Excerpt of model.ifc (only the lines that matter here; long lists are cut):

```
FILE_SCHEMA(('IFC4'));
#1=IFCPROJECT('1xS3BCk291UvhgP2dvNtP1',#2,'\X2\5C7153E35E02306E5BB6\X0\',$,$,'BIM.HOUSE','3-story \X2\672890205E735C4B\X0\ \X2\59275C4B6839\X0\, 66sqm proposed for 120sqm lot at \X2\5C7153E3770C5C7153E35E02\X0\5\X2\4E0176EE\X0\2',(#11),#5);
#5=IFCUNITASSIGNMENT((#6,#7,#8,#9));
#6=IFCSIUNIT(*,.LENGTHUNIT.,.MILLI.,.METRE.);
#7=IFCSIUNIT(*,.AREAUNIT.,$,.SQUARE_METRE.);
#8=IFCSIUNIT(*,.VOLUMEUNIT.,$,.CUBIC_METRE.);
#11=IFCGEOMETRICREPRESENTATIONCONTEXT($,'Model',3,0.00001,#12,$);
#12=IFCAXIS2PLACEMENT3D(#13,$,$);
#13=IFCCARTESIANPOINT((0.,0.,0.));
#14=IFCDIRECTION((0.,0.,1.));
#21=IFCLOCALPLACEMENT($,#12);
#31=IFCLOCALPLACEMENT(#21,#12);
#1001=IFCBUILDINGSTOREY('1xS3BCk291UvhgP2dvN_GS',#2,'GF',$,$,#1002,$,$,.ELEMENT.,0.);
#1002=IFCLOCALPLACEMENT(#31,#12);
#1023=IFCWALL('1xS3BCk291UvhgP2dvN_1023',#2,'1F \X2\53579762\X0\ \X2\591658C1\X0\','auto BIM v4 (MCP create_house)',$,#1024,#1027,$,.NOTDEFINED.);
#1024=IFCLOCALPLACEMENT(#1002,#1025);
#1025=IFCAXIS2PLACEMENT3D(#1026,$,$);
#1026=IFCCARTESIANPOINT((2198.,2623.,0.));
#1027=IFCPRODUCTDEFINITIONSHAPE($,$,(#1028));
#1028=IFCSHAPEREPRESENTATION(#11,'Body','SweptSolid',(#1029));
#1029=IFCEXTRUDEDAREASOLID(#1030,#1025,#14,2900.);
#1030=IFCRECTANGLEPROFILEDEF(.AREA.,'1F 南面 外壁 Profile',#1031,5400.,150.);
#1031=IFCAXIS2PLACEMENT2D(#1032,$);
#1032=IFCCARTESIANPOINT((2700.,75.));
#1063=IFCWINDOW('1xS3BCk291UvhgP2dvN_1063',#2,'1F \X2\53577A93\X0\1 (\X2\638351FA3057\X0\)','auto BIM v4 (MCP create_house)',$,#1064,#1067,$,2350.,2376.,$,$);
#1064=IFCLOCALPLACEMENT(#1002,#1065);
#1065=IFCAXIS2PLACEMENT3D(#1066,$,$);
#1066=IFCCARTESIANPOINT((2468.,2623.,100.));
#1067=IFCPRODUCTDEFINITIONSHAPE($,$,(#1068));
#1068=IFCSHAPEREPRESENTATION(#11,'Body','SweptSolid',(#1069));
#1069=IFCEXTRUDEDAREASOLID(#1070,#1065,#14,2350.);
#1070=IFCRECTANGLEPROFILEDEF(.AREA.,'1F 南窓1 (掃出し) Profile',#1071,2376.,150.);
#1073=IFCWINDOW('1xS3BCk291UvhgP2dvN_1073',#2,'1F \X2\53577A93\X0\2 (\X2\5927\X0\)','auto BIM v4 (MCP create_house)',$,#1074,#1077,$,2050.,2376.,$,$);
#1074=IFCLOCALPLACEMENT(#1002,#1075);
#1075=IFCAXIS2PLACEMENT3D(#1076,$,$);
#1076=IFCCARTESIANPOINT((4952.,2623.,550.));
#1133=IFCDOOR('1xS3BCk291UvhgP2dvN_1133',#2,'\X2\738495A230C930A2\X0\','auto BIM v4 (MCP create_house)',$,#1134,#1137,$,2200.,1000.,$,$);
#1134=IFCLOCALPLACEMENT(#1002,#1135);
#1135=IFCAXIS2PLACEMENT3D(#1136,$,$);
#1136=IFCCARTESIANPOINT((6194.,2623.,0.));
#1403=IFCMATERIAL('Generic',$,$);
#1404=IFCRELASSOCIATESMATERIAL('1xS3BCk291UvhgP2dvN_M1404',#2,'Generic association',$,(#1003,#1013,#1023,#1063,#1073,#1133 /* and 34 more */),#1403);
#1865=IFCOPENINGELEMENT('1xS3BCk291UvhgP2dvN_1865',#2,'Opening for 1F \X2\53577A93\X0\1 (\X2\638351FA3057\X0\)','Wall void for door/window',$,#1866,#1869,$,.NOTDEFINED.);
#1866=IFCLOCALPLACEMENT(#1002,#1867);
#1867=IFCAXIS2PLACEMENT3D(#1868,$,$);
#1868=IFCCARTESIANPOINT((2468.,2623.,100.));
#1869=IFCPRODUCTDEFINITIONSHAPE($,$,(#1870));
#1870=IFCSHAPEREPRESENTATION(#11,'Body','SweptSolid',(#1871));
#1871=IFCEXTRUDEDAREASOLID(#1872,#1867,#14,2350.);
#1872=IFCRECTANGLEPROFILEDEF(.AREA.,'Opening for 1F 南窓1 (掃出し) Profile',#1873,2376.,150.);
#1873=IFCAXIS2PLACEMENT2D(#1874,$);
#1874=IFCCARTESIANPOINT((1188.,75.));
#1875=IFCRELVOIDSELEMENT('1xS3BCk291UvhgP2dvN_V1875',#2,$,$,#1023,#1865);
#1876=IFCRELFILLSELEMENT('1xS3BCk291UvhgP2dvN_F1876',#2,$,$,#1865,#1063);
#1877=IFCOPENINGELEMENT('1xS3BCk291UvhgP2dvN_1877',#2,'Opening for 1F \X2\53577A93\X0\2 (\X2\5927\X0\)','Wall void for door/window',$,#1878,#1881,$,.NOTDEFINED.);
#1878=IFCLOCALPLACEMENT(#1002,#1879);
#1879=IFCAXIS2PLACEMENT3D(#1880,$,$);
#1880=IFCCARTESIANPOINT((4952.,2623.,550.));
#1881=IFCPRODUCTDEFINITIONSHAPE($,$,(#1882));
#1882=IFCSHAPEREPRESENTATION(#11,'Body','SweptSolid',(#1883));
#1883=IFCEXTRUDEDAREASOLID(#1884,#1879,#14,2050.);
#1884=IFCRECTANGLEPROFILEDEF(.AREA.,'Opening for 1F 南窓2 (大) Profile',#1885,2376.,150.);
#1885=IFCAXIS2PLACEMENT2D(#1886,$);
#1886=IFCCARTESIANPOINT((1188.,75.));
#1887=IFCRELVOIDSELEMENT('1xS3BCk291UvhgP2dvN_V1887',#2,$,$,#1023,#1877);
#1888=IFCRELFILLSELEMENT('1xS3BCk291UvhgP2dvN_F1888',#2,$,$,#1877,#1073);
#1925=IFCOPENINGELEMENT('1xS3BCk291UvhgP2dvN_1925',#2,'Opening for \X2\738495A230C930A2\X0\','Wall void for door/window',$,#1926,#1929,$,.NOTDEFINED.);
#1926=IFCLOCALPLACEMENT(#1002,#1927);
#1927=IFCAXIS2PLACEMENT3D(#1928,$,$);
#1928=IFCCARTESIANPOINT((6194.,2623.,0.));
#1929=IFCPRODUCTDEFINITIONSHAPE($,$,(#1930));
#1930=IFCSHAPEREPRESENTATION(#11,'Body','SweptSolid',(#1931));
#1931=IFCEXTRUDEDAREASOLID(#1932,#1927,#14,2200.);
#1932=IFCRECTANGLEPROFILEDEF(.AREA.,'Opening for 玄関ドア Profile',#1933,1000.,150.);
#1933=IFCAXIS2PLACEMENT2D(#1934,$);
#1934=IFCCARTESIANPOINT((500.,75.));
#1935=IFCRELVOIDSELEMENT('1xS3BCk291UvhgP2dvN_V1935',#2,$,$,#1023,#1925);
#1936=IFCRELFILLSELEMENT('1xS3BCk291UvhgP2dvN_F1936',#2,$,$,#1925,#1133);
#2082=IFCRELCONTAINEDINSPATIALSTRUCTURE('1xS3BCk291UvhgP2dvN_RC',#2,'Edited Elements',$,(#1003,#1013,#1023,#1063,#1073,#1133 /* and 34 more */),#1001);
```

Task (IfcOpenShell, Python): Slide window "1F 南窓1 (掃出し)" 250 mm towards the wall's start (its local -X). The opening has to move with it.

```python
import ifcopenshell
import ifcopenshell.api.geometry
import ifcopenshell.util.placement
import ifcopenshell.util.unit

model = ifcopenshell.open("model.ifc")
unit_scale = ifcopenshell.util.unit.calculate_unit_scale(model)

window = model.by_id(1063)
opening = window.FillsVoids[0].RelatingOpeningElement
wall = opening.VoidsElements[0].RelatingBuildingElement

wall_matrix = ifcopenshell.util.placement.get_local_placement(wall.ObjectPlacement)
shift = wall_matrix[:3, 0] * -0.25 / unit_scale
before = ifcopenshell.util.placement.get_local_placement(window.ObjectPlacement)[:3, 3].copy()

# The window is not placed relative to its opening, so move both.
for product in (opening, window):
    matrix = ifcopenshell.util.placement.get_local_placement(product.ObjectPlacement)
    matrix[:3, 3] += shift
    ifcopenshell.api.geometry.edit_object_placement(model, product=product, matrix=matrix, is_si=False)

after = ifcopenshell.util.placement.get_local_placement(window.ObjectPlacement)[:3, 3]
print("window moved by", (after - before).round(3) + 0.0)

model.write("model_updated.ifc")
```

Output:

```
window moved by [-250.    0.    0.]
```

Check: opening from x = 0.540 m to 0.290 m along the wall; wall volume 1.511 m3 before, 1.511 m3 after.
